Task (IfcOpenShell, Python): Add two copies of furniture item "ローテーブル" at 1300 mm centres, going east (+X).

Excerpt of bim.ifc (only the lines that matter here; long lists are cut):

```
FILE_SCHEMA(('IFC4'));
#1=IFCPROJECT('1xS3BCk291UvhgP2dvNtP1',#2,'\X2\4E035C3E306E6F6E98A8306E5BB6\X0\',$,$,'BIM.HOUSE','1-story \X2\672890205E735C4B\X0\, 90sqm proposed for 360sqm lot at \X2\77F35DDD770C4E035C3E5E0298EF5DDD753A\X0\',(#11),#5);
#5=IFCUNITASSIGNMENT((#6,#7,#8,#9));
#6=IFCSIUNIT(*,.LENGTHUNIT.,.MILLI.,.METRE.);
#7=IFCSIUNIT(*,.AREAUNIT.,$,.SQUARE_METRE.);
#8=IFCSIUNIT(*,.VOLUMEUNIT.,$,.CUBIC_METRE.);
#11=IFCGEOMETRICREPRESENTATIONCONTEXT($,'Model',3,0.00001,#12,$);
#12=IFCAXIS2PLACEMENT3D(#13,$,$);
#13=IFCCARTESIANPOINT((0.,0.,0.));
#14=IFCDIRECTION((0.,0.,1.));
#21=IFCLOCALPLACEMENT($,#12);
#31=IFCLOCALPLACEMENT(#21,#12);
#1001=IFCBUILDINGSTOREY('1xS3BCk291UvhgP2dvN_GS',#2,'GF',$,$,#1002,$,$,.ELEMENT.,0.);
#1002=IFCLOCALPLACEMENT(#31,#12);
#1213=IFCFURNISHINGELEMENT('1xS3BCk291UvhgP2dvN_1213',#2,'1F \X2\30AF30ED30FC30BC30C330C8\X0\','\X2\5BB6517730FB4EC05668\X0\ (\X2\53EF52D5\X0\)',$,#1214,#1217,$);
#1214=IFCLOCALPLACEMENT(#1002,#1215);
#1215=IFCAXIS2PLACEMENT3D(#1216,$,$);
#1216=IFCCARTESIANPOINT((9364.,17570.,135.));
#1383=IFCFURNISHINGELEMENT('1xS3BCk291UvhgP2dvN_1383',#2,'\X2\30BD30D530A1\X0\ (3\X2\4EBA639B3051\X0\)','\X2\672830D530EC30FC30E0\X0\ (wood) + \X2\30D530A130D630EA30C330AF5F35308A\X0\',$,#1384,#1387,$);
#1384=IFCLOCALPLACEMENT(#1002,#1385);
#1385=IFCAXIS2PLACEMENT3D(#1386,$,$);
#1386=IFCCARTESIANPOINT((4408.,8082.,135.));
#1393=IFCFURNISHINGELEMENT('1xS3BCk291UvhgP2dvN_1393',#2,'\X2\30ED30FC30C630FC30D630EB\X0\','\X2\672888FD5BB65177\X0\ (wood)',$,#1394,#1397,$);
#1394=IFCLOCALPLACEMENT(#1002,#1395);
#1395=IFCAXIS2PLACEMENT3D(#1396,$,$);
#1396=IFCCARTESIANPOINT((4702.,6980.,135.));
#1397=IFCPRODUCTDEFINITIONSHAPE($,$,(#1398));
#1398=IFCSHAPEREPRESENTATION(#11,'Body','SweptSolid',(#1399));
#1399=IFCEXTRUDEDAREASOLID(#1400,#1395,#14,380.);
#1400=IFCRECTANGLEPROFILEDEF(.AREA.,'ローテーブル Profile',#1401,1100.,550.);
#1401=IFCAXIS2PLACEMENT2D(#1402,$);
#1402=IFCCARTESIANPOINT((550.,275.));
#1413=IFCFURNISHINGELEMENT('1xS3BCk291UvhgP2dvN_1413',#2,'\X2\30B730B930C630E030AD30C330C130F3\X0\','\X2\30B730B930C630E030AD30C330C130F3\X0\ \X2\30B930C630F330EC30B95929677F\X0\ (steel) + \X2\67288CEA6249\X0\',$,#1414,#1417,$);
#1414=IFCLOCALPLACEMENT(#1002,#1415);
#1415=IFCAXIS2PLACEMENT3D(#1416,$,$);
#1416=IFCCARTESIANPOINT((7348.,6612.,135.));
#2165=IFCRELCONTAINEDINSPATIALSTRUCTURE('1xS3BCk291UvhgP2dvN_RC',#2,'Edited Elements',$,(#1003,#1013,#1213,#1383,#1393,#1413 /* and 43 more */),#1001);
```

```python
import numpy as np
import ifcopenshell
import ifcopenshell.api.geometry
import ifcopenshell.api.root
import ifcopenshell.util.element
import ifcopenshell.util.placement
import ifcopenshell.util.unit

model = ifcopenshell.open("bim.ifc")
unit_scale = ifcopenshell.util.unit.calculate_unit_scale(model)


def reuse_history(source, copy):
    """copy_class also copies each property set's owner history, people and application; keep the originals."""
    for rel in copy.IsDefinedBy:
        if rel.is_a("IfcRelDefinesByProperties") and (history := rel.RelatingPropertyDefinition.OwnerHistory):
            rel.RelatingPropertyDefinition.OwnerHistory = source.OwnerHistory
            ifcopenshell.util.element.remove_deep2(model, history)


source = model.by_id(1393)
base = ifcopenshell.util.placement.get_local_placement(source.ObjectPlacement)
step = np.array([1.0, 0.0, 0.0]) * 1.3 / unit_scale

for i in range(1, 3):
    copy = ifcopenshell.api.root.copy_class(model, product=source)
    copy.Representation = ifcopenshell.util.element.copy_deep(
        model, source.Representation, exclude=["IfcGeometricRepresentationContext", "IfcRepresentationMap"]
    )
    reuse_history(source, copy)
    matrix = base.copy()
    matrix[:3, 3] += i * step
    print("added at", matrix[:3, 3].round(3) + 0.0)
    ifcopenshell.api.geometry.edit_object_placement(model, product=copy, matrix=matrix, is_si=False)

model.write("bim_updated.ifc")
```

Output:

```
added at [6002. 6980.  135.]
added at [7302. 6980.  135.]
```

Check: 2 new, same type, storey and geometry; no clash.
